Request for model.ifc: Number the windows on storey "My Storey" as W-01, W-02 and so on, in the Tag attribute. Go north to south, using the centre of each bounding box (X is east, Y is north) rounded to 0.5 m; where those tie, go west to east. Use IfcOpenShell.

First a look at what the model holds.

```python
import ifcopenshell
import ifcopenshell.util.element
import ifcopenshell.util.placement

model = ifcopenshell.open("model.ifc")
print(model.schema)
storey = next(s for s in model.by_type("IfcBuildingStorey") if s.Name == "My Storey")
windows = [e for e in ifcopenshell.util.element.get_decomposition(storey) if e.is_a("IfcWindow")]
for e in sorted(windows, key=lambda e: e.id()):
    origin = ifcopenshell.util.placement.get_local_placement(e.ObjectPlacement)[:3, 3]
    print(e.id(), e.Tag, e.Name, origin.round(2) + 0.0, sep=" | ")
```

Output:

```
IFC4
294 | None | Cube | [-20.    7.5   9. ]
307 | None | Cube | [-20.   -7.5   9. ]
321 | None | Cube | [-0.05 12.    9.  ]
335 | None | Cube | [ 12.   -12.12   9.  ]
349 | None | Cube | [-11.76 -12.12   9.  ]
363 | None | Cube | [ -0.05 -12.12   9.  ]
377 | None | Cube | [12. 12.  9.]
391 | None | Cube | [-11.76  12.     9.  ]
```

```python
import ifcopenshell
import ifcopenshell.geom
import ifcopenshell.util.element
import ifcopenshell.util.shape

model = ifcopenshell.open("model.ifc")
settings = ifcopenshell.geom.settings()
settings.set("use-world-coords", True)


def centre(element):
    shape = ifcopenshell.geom.create_shape(settings, element)
    return ifcopenshell.util.shape.get_bbox_centroid(shape.geometry)


storey = next(s for s in model.by_type("IfcBuildingStorey") if s.Name == "My Storey")
windows = [e for e in ifcopenshell.util.element.get_decomposition(storey) if e.is_a("IfcWindow")]

# Insertion points can sit at a corner or the storey origin, so sort by the geometry (in metres).
centres = {e: centre(e) for e in windows}
windows.sort(key=lambda e: (-round(centres[e][1] / 0.5), centres[e][0]))

for i, e in enumerate(windows, start=1):
    number = f"W-{i:02d}"
    e.Tag = number
    print(e.id(), number)

model.write("model_rev.ifc")
```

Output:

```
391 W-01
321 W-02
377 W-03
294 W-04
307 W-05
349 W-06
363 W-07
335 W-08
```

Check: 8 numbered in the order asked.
